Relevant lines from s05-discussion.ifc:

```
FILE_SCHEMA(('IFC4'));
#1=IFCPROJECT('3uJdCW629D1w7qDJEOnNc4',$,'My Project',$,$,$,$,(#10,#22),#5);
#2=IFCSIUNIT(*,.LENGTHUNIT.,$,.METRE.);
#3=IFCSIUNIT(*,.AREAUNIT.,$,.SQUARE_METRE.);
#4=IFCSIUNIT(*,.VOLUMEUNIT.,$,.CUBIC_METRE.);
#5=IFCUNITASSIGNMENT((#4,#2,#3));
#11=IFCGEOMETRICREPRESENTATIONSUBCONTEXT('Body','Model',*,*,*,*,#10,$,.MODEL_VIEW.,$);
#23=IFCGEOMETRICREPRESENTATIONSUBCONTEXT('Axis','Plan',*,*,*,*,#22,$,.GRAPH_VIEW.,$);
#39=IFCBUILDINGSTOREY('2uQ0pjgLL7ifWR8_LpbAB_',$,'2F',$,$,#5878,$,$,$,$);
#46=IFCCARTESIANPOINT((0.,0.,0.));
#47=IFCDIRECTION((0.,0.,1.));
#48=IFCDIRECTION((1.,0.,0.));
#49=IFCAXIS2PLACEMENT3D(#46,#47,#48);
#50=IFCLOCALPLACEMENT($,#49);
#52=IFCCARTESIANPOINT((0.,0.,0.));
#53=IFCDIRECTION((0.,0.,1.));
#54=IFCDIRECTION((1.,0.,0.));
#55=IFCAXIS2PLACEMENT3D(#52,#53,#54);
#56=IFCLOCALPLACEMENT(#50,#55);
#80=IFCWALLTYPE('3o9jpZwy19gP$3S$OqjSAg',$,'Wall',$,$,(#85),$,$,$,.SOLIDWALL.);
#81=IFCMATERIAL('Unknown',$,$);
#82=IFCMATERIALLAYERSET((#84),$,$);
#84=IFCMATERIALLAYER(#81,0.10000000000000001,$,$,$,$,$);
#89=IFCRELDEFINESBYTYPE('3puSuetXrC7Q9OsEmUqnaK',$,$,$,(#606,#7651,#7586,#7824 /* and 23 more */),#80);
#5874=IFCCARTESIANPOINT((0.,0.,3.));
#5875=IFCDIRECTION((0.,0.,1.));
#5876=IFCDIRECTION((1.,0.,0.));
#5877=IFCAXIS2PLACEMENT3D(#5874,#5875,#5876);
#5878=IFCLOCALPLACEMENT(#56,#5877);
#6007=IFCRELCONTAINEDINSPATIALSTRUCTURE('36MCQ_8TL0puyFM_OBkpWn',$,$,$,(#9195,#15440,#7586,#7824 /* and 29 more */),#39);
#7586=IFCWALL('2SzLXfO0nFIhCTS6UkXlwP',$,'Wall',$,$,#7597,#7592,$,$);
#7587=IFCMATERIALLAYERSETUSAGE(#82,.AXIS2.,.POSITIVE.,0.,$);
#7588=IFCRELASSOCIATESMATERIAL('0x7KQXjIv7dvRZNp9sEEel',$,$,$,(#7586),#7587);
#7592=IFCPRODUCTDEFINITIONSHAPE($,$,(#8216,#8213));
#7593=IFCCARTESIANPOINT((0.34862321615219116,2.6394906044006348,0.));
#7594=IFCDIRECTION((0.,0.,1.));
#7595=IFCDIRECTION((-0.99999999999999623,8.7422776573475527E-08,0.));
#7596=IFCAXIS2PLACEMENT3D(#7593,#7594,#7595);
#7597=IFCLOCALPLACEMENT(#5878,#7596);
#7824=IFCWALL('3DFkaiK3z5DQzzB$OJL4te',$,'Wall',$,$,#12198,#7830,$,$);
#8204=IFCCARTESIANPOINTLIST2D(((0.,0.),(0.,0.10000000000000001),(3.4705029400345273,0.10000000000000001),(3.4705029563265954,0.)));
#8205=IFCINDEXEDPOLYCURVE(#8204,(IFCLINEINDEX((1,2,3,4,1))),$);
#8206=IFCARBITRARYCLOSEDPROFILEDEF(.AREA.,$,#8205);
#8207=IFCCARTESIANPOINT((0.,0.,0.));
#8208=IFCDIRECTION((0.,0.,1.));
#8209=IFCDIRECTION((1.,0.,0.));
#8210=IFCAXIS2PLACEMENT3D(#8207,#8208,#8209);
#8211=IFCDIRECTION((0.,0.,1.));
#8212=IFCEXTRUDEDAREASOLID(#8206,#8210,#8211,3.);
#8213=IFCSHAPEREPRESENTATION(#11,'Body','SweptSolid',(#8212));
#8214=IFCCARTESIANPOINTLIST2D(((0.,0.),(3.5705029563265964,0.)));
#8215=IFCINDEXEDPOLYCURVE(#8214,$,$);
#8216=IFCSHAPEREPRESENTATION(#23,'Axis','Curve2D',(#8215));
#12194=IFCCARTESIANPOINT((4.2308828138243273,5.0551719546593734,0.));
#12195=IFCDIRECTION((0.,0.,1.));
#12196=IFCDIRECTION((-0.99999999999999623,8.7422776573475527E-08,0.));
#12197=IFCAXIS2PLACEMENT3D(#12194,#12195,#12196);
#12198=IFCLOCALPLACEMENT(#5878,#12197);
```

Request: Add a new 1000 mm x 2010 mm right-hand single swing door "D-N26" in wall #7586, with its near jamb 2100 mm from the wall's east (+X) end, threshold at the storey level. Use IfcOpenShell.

```python
import numpy as np
import ifcopenshell
import ifcopenshell.api.feature
import ifcopenshell.api.geometry
import ifcopenshell.api.root
import ifcopenshell.api.spatial
import ifcopenshell.geom
import ifcopenshell.util.element
import ifcopenshell.util.placement
import ifcopenshell.util.representation
import ifcopenshell.util.shape
import ifcopenshell.util.unit

model = ifcopenshell.open("s05-discussion.ifc")
unit_scale = ifcopenshell.util.unit.calculate_unit_scale(model)
settings = ifcopenshell.geom.settings()


def volume(element):
    """Net volume in cubic metres, openings subtracted."""
    shape = ifcopenshell.geom.create_shape(settings, element)
    return ifcopenshell.util.shape.get_volume(shape.geometry)


wall = model.by_guid("2SzLXfO0nFIhCTS6UkXlwP")
storey = ifcopenshell.util.element.get_container(wall, ifc_class="IfcBuildingStorey")
context = ifcopenshell.util.representation.get_context(model, "Model", "Body", "MODEL_VIEW")
before = volume(wall)

width, height, from_end, sill = 1, 2.01, 2.1, 0.0  # metres

# The wall runs along its own X axis, and the end named is its -X end.
wall_shape = ifcopenshell.geom.create_shape(settings, wall)
x, y, z = ifcopenshell.util.shape.get_vertices(wall_shape.geometry).T
start = x.min() + from_end
face, thickness = float(y.min()), float(y.max() - y.min())
wall_matrix = ifcopenshell.util.placement.get_local_placement(wall.ObjectPlacement)
level = ifcopenshell.util.placement.get_local_placement(storey.ObjectPlacement)[2, 3]


def in_wall(x, y):
    """Placement at x, y metres in the wall's axes, at sill height."""
    matrix = wall_matrix.copy()
    matrix[:, 3] = wall_matrix @ np.array([x / unit_scale, y / unit_scale, 0.0, 1.0])
    matrix[2, 3] = level + sill / unit_scale
    return matrix


# Opening: a box that overshoots both wall faces by 50 mm.
opening = ifcopenshell.api.root.create_entity(model, ifc_class="IfcOpeningElement", predefined_type="OPENING")
box = ifcopenshell.api.geometry.add_wall_representation(
    model, context=context, length=width, height=height, thickness=thickness + 0.1
)
ifcopenshell.api.geometry.assign_representation(model, product=opening, representation=box)
ifcopenshell.api.geometry.edit_object_placement(model, product=opening, matrix=in_wall(start, face - 0.05), is_si=False)
ifcopenshell.api.feature.add_feature(model, feature=opening, element=wall)

door = ifcopenshell.api.root.create_entity(model, ifc_class="IfcDoor", name="D-N26", predefined_type="DOOR")
door.OverallWidth, door.OverallHeight = width / unit_scale, height / unit_scale
door.OperationType = "SINGLE_SWING_RIGHT"
body = ifcopenshell.api.geometry.add_door_representation(
    model,
    context=context,
    overall_width=door.OverallWidth,
    overall_height=door.OverallHeight,
    operation_type="SINGLE_SWING_RIGHT",
    lining_properties={"LiningDepth": thickness / unit_scale, "ThresholdDepth": thickness / unit_scale},
)
ifcopenshell.api.geometry.assign_representation(model, product=door, representation=body)
ifcopenshell.api.spatial.assign_container(model, products=[door], relating_structure=storey)
ifcopenshell.api.feature.add_filling(model, opening=opening, element=door)

# The lining spans the wall, so the door starts at the wall face.
ifcopenshell.api.geometry.edit_object_placement(model, product=door, matrix=in_wall(start, face), is_si=False)

after = volume(wall)

print(f"wall volume {before:.3f} -> {after:.3f} m3")

model.write("s05-discussion_updated.ifc")
```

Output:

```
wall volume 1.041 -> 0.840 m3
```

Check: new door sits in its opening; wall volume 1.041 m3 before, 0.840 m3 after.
